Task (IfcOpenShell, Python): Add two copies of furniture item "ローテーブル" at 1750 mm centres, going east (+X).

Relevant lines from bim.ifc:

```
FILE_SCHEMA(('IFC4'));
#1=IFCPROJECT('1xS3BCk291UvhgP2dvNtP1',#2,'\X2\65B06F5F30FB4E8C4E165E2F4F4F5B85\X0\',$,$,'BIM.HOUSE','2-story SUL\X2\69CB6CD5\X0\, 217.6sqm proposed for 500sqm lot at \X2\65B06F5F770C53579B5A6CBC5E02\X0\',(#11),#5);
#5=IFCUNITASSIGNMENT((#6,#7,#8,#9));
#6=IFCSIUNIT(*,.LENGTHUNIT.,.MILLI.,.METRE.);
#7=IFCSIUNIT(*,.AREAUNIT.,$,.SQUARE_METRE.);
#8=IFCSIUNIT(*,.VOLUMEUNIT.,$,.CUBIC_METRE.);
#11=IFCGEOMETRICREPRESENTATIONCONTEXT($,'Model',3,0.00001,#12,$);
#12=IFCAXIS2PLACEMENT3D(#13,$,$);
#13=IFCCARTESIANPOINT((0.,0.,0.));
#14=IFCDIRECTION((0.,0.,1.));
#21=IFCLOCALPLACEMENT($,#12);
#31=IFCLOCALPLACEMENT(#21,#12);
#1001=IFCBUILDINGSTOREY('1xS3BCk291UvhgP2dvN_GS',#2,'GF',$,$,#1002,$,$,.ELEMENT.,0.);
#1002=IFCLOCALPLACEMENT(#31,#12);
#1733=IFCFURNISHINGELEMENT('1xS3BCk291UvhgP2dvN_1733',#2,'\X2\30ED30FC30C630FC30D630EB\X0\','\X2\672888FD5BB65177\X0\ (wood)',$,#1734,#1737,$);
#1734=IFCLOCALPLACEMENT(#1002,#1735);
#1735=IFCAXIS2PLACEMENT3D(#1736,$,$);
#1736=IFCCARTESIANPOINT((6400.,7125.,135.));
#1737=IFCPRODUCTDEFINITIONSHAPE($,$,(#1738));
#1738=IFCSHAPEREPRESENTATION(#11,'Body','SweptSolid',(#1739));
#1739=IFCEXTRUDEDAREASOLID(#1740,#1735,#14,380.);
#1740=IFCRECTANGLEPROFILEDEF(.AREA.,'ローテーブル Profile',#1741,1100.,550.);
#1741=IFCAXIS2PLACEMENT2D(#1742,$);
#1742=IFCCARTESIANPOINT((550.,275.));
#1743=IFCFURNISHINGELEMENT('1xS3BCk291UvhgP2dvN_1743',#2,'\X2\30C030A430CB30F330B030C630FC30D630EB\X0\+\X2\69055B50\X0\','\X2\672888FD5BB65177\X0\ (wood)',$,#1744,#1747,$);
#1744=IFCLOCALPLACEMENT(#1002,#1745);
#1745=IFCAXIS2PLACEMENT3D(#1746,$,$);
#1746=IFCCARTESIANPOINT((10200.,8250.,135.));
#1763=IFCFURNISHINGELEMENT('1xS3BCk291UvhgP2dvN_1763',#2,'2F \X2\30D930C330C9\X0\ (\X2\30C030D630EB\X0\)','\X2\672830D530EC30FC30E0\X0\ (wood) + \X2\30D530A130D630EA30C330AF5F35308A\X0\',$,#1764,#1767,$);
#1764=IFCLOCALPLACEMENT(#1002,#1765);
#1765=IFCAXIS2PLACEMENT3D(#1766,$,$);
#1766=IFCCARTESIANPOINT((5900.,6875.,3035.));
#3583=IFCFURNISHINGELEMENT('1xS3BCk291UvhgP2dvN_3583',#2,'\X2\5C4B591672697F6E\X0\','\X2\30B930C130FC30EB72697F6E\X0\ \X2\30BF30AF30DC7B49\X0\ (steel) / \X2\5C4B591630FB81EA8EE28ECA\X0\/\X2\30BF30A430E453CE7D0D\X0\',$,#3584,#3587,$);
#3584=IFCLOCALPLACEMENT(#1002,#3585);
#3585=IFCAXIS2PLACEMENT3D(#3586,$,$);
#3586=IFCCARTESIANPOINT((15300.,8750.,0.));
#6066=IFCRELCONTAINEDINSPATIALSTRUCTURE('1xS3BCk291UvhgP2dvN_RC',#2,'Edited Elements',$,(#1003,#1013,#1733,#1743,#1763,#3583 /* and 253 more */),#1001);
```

```python
import numpy as np
import ifcopenshell
import ifcopenshell.api.geometry
import ifcopenshell.api.root
import ifcopenshell.util.element
import ifcopenshell.util.placement
import ifcopenshell.util.unit

model = ifcopenshell.open("bim.ifc")
unit_scale = ifcopenshell.util.unit.calculate_unit_scale(model)


def reuse_history(source, copy):
    """copy_class also copies each property set's owner history, people and application; keep the originals."""
    for rel in copy.IsDefinedBy:
        if rel.is_a("IfcRelDefinesByProperties") and (history := rel.RelatingPropertyDefinition.OwnerHistory):
            rel.RelatingPropertyDefinition.OwnerHistory = source.OwnerHistory
            ifcopenshell.util.element.remove_deep2(model, history)


source = model.by_guid("1xS3BCk291UvhgP2dvN_1733")
base = ifcopenshell.util.placement.get_local_placement(source.ObjectPlacement)
step = np.array([1.0, 0.0, 0.0]) * 1.75 / unit_scale

for i in range(1, 3):
    copy = ifcopenshell.api.root.copy_class(model, product=source)
    copy.Representation = ifcopenshell.util.element.copy_deep(
        model, source.Representation, exclude=["IfcGeometricRepresentationContext", "IfcRepresentationMap"]
    )
    reuse_history(source, copy)
    matrix = base.copy()
    matrix[:3, 3] += i * step
    print("added at", matrix[:3, 3].round(3) + 0.0)
    ifcopenshell.api.geometry.edit_object_placement(model, product=copy, matrix=matrix, is_si=False)

model.write("bim_rev.ifc")
```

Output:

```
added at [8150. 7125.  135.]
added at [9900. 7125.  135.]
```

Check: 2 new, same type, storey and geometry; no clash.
